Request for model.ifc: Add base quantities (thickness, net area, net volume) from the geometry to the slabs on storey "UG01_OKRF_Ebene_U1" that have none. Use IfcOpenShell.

First a look at what the model holds.

```python
import ifcopenshell
import ifcopenshell.util.element
import ifcopenshell.util.unit

model = ifcopenshell.open("model.ifc")
print(model.schema)
for unit_type in ("LENGTHUNIT", "AREAUNIT", "VOLUMEUNIT"):
    print(unit_type, ifcopenshell.util.unit.calculate_unit_scale(model, unit_type))
storey = next(s for s in model.by_type("IfcBuildingStorey") if s.Name == "UG01_OKRF_Ebene_U1")
slabs = [e for e in ifcopenshell.util.element.get_decomposition(storey) if e.is_a("IfcSlab")]
for e in sorted(slabs, key=lambda e: e.id()):
    print(e.id(), e.is_a(), e.Name, list(ifcopenshell.util.element.get_psets(e, qtos_only=True)), sep=" | ")
```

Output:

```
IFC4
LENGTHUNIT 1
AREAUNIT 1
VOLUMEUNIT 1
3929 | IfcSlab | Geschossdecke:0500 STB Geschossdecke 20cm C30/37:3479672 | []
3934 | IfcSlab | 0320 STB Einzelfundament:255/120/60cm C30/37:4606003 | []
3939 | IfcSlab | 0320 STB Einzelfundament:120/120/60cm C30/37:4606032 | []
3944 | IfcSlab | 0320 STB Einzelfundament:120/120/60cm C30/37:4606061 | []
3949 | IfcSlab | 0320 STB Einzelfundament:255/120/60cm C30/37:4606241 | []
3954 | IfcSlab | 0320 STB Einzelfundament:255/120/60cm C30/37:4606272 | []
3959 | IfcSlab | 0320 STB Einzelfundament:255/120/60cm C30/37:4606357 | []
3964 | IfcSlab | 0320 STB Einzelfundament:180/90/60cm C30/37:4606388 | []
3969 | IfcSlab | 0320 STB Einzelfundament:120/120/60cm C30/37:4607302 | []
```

```python
import ifcopenshell
import ifcopenshell.api.pset
import ifcopenshell.geom
import ifcopenshell.util.element
import ifcopenshell.util.shape
import ifcopenshell.util.unit

model = ifcopenshell.open("model.ifc")
unit_scale = ifcopenshell.util.unit.calculate_unit_scale(model)
area_scale = ifcopenshell.util.unit.calculate_unit_scale(model, "AREAUNIT")
volume_scale = ifcopenshell.util.unit.calculate_unit_scale(model, "VOLUMEUNIT")
settings = ifcopenshell.geom.settings()

storey = next(s for s in model.by_type("IfcBuildingStorey") if s.Name == "UG01_OKRF_Ebene_U1")
slabs = [e for e in ifcopenshell.util.element.get_decomposition(storey) if e.is_a("IfcSlab")]

for e in sorted(slabs, key=lambda e: e.id()):
    if ifcopenshell.util.element.get_psets(e, qtos_only=True, should_inherit=False):
        continue
    # Geometry comes back in metres, in the element's own axes.
    shape = ifcopenshell.geom.create_shape(settings, e)
    values = {
        "Width": ifcopenshell.util.shape.get_z(shape.geometry) / unit_scale,
        "NetArea": ifcopenshell.util.shape.get_footprint_area(shape.geometry) / area_scale,
        "NetVolume": ifcopenshell.util.shape.get_volume(shape.geometry) / volume_scale,
    }
    qto = ifcopenshell.api.pset.add_qto(model, product=e, name="Qto_SlabBaseQuantities")
    ifcopenshell.api.pset.edit_qto(model, qto=qto, properties=values)
    print(e.id(), {k: round(v, 3) for k, v in values.items()})

model.write("model_edited.ifc")
```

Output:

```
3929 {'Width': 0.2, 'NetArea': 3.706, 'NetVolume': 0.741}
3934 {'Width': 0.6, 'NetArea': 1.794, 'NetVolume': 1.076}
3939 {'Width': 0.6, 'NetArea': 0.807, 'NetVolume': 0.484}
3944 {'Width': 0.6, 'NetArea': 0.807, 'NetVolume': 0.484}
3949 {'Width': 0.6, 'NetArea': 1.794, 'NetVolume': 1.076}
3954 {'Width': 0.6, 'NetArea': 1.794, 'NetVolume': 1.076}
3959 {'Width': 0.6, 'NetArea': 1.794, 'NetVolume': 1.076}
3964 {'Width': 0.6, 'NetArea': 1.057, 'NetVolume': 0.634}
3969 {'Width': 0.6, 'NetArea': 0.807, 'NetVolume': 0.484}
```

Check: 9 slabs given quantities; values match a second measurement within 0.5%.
